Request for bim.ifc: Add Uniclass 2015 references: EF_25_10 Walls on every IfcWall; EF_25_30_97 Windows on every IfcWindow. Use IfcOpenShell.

First a look at what the model holds.

```python
import ifcopenshell

model = ifcopenshell.open("bim.ifc")
print(model.schema)
print("classifications:", [c.Name for c in model.by_type("IfcClassification")])
for ifc_class in ("IfcDoor", "IfcRoof", "IfcStair", "IfcWall", "IfcWindow"):
    print(ifc_class, len(model.by_type(ifc_class)))
```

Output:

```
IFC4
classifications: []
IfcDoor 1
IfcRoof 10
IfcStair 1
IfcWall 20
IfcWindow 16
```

```python
import ifcopenshell
import ifcopenshell.api.classification

model = ifcopenshell.open("bim.ifc")

system = ifcopenshell.api.classification.add_classification(model, classification="Uniclass 2015")

codes = {
    "IfcWall": ("EF_25_10", "Walls"),
    "IfcWindow": ("EF_25_30_97", "Windows"),
}
for ifc_class, (code, name) in codes.items():
    products = model.by_type(ifc_class)
    ifcopenshell.api.classification.add_reference(
        model, products=products, classification=system, identification=code, name=name
    )
    print(code, len(products))

model.write("bim_updated.ifc")
```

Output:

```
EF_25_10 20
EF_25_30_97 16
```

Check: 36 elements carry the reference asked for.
